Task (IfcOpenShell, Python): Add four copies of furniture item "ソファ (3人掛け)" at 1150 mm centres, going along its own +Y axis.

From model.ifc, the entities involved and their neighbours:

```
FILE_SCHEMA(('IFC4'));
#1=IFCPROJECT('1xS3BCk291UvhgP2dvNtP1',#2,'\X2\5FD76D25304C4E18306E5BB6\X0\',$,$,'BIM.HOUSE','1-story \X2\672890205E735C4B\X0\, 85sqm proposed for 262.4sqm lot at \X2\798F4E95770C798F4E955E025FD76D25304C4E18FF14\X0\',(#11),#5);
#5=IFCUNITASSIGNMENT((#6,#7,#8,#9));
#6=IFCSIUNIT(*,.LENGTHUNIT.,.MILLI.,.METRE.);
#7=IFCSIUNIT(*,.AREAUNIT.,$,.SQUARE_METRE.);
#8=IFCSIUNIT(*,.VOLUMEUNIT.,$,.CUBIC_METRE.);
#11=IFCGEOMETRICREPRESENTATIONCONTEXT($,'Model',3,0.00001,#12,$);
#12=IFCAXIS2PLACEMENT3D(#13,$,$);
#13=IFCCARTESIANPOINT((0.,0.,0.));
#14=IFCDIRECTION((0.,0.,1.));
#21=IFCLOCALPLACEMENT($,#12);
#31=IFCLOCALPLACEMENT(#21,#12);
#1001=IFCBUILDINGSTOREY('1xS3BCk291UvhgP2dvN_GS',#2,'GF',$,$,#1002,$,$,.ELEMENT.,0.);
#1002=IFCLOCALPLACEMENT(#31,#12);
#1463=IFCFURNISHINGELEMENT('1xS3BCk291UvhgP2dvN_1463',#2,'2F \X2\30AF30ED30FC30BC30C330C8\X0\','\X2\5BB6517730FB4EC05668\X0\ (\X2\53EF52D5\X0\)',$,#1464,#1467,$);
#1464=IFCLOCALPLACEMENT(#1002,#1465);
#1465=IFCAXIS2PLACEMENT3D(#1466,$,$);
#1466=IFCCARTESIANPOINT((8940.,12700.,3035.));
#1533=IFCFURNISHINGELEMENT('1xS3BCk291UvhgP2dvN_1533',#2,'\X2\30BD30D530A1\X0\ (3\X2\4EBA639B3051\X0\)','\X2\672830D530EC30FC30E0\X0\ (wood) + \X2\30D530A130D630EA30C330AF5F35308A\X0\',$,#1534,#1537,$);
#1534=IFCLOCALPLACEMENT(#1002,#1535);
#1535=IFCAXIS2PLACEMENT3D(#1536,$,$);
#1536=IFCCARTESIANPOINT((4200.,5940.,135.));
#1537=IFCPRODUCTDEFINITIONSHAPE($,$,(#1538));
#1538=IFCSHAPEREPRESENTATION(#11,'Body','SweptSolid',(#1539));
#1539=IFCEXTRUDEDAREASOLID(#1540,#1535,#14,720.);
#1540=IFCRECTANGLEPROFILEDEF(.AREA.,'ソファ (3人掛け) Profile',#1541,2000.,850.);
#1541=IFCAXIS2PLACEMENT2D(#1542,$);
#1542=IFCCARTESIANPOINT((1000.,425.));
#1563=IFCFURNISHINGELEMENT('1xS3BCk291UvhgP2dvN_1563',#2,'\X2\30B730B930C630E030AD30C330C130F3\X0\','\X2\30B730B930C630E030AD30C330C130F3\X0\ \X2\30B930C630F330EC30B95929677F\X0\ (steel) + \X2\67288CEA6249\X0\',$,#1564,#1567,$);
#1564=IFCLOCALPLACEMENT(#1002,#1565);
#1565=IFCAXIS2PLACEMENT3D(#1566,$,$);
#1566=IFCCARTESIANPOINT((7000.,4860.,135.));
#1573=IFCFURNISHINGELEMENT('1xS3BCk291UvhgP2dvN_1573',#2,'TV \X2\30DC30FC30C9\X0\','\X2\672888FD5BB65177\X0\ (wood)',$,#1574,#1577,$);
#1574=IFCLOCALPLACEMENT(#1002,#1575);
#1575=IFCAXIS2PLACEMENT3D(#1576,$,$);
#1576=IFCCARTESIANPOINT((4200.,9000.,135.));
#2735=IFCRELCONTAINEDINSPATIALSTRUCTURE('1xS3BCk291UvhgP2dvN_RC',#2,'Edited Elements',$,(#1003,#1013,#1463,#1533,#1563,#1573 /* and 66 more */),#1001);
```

```python
import ifcopenshell
import ifcopenshell.api.geometry
import ifcopenshell.api.root
import ifcopenshell.util.element
import ifcopenshell.util.placement

model = ifcopenshell.open("model.ifc")


def reuse_history(source, copy):
    """copy_class also copies each property set's owner history, people and application; keep the originals."""
    for rel in copy.IsDefinedBy:
        if rel.is_a("IfcRelDefinesByProperties") and (history := rel.RelatingPropertyDefinition.OwnerHistory):
            rel.RelatingPropertyDefinition.OwnerHistory = source.OwnerHistory
            ifcopenshell.util.element.remove_deep2(model, history)


source = model.by_guid("1xS3BCk291UvhgP2dvN_1533")
base = ifcopenshell.util.placement.get_local_placement(source.ObjectPlacement)
step = base[:3, 1] * 1150.0

for i in range(1, 5):
    copy = ifcopenshell.api.root.copy_class(model, product=source)
    copy.Representation = ifcopenshell.util.element.copy_deep(
        model, source.Representation, exclude=["IfcGeometricRepresentationContext", "IfcRepresentationMap"]
    )
    reuse_history(source, copy)
    matrix = base.copy()
    matrix[:3, 3] += i * step
    print("added at", matrix[:3, 3].round(3) + 0.0)
    ifcopenshell.api.geometry.edit_object_placement(model, product=copy, matrix=matrix, is_si=False)

model.write("model_edited.ifc")
```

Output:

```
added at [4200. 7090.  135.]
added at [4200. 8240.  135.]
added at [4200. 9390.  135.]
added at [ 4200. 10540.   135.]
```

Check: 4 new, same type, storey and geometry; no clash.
